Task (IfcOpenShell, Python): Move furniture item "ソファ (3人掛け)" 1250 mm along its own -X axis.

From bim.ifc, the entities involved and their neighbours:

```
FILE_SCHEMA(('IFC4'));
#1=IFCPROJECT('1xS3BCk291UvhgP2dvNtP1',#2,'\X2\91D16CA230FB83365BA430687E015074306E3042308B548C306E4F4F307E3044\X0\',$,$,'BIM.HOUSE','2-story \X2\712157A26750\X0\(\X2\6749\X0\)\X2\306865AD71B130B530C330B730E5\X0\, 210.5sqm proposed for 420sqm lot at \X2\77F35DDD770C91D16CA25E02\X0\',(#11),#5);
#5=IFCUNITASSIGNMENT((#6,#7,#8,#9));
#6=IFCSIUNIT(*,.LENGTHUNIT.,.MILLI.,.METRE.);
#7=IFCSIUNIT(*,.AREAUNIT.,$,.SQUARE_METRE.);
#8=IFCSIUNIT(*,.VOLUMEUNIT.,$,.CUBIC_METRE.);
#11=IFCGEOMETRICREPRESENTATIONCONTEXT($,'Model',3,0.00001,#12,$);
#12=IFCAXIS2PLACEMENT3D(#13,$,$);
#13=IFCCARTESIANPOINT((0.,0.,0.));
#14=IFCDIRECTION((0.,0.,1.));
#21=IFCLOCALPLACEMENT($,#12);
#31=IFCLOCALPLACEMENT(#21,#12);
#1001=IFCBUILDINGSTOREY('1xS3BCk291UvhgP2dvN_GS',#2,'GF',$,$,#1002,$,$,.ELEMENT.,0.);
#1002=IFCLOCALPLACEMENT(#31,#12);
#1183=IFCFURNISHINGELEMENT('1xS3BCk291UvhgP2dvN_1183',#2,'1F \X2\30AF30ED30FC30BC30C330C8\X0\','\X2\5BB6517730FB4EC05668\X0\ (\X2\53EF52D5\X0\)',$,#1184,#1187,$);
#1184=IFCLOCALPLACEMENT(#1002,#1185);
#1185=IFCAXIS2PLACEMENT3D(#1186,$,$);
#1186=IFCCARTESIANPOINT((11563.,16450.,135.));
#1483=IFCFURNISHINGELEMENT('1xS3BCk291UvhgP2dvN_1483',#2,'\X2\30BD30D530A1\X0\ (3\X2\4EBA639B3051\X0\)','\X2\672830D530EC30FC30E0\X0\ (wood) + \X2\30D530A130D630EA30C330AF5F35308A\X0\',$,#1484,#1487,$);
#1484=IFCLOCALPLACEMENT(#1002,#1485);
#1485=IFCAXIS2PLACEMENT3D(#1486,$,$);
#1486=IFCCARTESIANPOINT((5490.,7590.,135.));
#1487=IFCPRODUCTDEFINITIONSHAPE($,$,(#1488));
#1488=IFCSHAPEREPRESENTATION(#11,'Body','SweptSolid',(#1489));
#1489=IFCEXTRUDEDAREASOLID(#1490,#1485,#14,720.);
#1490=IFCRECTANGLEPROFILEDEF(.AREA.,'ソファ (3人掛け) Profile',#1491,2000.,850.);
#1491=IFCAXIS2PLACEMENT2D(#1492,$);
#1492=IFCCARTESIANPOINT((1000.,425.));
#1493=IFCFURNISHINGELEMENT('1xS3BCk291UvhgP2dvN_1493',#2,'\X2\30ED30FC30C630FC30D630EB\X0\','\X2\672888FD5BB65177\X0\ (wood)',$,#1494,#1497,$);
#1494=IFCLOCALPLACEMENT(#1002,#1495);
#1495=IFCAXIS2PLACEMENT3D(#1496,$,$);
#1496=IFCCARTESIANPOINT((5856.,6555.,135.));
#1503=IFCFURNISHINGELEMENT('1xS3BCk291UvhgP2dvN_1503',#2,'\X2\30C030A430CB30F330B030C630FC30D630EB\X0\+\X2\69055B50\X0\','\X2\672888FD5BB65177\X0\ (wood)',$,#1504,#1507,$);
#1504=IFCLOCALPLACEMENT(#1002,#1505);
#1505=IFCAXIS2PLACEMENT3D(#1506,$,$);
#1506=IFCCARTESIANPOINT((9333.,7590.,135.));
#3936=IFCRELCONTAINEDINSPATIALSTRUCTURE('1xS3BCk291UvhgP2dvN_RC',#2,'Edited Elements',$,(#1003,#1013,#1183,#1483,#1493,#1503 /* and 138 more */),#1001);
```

```python
import ifcopenshell
import ifcopenshell.api.geometry
import ifcopenshell.util.placement
import ifcopenshell.util.unit

model = ifcopenshell.open("bim.ifc")
unit_scale = ifcopenshell.util.unit.calculate_unit_scale(model)

item = model.by_guid("1xS3BCk291UvhgP2dvN_1483")
matrix = ifcopenshell.util.placement.get_local_placement(item.ObjectPlacement)
matrix[:3, 3] -= matrix[:3, 0] * 1.25 / unit_scale
ifcopenshell.api.geometry.edit_object_placement(model, product=item, matrix=matrix, is_si=False)

print(ifcopenshell.util.placement.get_local_placement(item.ObjectPlacement).round(3) + 0.0)

model.write("bim-out.ifc")
```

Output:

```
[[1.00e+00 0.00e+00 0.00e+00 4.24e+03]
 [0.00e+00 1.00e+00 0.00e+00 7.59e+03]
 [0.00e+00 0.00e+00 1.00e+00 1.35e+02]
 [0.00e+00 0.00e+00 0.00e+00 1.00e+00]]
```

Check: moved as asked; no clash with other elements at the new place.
